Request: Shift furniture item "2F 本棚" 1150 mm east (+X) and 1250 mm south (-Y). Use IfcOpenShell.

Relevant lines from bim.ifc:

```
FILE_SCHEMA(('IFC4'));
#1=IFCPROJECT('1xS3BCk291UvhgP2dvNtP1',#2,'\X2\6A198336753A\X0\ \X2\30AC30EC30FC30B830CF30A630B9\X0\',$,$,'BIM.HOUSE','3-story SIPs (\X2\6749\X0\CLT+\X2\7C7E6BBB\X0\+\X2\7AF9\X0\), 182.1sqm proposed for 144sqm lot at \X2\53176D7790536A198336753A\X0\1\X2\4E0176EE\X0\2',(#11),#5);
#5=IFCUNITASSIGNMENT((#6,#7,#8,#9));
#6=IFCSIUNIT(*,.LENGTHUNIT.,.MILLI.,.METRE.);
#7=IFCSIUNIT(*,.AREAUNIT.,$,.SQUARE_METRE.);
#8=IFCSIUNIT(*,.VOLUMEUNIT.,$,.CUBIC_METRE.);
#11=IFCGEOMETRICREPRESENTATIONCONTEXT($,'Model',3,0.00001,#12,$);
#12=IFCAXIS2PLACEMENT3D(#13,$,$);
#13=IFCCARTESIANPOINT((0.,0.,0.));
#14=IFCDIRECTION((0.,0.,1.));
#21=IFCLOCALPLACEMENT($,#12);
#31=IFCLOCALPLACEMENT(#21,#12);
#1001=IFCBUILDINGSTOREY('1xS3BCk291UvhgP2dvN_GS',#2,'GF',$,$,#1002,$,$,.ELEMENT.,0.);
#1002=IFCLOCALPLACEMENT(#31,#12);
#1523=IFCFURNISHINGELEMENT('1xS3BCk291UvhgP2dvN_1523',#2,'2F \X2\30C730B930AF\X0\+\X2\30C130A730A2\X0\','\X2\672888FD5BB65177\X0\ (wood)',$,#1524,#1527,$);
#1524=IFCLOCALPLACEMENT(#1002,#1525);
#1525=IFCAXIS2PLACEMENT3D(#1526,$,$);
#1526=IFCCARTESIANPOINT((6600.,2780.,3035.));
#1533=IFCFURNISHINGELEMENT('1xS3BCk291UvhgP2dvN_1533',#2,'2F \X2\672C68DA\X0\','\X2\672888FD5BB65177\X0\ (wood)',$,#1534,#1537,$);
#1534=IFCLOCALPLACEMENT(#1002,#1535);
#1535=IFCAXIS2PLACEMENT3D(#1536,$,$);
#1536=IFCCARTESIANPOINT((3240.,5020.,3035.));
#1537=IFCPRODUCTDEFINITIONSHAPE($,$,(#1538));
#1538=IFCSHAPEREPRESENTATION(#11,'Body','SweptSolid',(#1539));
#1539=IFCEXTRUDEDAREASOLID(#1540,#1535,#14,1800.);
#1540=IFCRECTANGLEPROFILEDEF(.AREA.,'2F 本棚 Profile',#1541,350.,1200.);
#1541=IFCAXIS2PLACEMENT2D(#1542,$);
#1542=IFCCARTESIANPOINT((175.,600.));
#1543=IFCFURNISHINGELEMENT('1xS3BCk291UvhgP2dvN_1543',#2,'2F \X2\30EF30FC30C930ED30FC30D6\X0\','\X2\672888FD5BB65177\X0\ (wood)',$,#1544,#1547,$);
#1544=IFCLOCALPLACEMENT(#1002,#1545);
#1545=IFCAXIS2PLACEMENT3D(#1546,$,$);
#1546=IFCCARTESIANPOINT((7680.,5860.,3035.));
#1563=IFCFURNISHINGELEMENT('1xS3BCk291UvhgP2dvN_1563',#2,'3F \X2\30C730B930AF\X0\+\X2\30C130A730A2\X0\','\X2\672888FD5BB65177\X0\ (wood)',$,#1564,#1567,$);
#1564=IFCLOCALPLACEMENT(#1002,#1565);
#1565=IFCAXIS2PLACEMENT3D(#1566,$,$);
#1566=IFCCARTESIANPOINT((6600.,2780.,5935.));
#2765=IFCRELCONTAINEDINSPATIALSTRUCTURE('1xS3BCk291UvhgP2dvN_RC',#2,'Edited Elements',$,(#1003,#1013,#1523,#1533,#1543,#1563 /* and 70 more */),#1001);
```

```python
import ifcopenshell
import ifcopenshell.api.geometry
import ifcopenshell.util.placement
import ifcopenshell.util.unit

model = ifcopenshell.open("bim.ifc")
unit_scale = ifcopenshell.util.unit.calculate_unit_scale(model)

item = model.by_guid("1xS3BCk291UvhgP2dvN_1533")
matrix = ifcopenshell.util.placement.get_local_placement(item.ObjectPlacement)
matrix[0, 3] += 1.15 / unit_scale
matrix[1, 3] -= 1.25 / unit_scale
ifcopenshell.api.geometry.edit_object_placement(model, product=item, matrix=matrix, is_si=False)

print(ifcopenshell.util.placement.get_local_placement(item.ObjectPlacement).round(3) + 0.0)

model.write("bim_v2.ifc")
```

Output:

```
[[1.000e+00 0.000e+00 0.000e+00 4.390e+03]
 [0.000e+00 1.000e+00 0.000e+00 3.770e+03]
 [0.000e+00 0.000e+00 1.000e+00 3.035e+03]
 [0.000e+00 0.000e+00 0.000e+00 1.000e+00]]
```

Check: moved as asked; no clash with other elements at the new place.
